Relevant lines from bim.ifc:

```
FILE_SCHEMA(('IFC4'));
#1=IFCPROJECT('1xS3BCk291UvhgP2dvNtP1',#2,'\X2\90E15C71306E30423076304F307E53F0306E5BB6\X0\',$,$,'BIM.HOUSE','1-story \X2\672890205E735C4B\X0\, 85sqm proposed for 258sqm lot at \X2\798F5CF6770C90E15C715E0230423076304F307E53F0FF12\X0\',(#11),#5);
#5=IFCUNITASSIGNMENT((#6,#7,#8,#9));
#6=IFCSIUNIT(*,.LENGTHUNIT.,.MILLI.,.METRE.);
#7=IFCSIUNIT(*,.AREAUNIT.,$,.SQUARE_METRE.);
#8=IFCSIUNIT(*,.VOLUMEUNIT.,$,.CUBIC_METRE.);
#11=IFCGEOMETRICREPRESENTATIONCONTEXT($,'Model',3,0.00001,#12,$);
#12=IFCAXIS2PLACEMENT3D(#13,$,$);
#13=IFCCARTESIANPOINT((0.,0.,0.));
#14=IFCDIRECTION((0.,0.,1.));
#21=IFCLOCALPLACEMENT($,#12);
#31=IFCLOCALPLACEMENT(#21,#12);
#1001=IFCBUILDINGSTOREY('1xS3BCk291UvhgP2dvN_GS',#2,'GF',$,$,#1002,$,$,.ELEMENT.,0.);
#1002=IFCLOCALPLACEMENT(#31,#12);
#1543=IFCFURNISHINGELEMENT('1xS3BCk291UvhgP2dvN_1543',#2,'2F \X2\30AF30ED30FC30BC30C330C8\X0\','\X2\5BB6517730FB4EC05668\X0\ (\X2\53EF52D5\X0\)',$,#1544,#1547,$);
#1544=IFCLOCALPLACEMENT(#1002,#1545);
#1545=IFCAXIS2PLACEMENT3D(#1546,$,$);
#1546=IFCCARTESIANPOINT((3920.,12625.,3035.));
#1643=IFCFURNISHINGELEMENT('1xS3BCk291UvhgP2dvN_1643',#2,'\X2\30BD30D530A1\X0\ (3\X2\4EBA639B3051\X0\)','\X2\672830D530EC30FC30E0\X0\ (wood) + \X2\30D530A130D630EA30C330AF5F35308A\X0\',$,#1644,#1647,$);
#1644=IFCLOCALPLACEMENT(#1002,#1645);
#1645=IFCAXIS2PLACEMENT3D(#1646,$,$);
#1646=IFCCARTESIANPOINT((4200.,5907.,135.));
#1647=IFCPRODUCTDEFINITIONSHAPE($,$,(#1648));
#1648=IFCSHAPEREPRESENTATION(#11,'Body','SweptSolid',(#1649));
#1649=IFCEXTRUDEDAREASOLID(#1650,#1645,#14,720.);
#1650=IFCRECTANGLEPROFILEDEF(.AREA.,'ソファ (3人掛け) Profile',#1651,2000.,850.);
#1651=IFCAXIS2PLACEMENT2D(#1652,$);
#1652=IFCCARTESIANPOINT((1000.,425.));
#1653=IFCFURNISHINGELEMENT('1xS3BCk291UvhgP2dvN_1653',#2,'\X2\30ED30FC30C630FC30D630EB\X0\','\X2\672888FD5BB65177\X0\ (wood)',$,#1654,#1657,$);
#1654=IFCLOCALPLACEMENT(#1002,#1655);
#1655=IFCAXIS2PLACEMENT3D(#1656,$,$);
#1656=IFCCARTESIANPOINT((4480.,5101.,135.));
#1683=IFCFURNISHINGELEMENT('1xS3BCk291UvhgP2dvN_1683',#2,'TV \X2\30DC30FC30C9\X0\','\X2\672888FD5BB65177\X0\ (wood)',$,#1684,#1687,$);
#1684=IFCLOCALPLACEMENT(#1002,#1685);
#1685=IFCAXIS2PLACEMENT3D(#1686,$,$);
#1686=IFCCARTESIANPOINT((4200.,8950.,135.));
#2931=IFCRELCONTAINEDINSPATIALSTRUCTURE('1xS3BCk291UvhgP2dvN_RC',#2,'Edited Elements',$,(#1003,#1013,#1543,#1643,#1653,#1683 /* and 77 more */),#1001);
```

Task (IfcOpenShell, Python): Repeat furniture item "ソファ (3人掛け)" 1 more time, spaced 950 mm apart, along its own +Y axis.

```python
import ifcopenshell
import ifcopenshell.api.geometry
import ifcopenshell.api.root
import ifcopenshell.util.element
import ifcopenshell.util.placement
import ifcopenshell.util.unit

model = ifcopenshell.open("bim.ifc")
unit_scale = ifcopenshell.util.unit.calculate_unit_scale(model)


def reuse_history(source, copy):
    """copy_class also copies each property set's owner history, people and application; keep the originals."""
    for rel in copy.IsDefinedBy:
        if rel.is_a("IfcRelDefinesByProperties") and (history := rel.RelatingPropertyDefinition.OwnerHistory):
            rel.RelatingPropertyDefinition.OwnerHistory = source.OwnerHistory
            ifcopenshell.util.element.remove_deep2(model, history)


source = model.by_guid("1xS3BCk291UvhgP2dvN_1643")
base = ifcopenshell.util.placement.get_local_placement(source.ObjectPlacement)
step = base[:3, 1] * 0.95 / unit_scale

for i in range(1, 2):
    copy = ifcopenshell.api.root.copy_class(model, product=source)
    copy.Representation = ifcopenshell.util.element.copy_deep(
        model, source.Representation, exclude=["IfcGeometricRepresentationContext", "IfcRepresentationMap"]
    )
    reuse_history(source, copy)
    matrix = base.copy()
    matrix[:3, 3] += i * step
    print("added at", matrix[:3, 3].round(3) + 0.0)
    ifcopenshell.api.geometry.edit_object_placement(model, product=copy, matrix=matrix, is_si=False)

model.write("bim_updated.ifc")
```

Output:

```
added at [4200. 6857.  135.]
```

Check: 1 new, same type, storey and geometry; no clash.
